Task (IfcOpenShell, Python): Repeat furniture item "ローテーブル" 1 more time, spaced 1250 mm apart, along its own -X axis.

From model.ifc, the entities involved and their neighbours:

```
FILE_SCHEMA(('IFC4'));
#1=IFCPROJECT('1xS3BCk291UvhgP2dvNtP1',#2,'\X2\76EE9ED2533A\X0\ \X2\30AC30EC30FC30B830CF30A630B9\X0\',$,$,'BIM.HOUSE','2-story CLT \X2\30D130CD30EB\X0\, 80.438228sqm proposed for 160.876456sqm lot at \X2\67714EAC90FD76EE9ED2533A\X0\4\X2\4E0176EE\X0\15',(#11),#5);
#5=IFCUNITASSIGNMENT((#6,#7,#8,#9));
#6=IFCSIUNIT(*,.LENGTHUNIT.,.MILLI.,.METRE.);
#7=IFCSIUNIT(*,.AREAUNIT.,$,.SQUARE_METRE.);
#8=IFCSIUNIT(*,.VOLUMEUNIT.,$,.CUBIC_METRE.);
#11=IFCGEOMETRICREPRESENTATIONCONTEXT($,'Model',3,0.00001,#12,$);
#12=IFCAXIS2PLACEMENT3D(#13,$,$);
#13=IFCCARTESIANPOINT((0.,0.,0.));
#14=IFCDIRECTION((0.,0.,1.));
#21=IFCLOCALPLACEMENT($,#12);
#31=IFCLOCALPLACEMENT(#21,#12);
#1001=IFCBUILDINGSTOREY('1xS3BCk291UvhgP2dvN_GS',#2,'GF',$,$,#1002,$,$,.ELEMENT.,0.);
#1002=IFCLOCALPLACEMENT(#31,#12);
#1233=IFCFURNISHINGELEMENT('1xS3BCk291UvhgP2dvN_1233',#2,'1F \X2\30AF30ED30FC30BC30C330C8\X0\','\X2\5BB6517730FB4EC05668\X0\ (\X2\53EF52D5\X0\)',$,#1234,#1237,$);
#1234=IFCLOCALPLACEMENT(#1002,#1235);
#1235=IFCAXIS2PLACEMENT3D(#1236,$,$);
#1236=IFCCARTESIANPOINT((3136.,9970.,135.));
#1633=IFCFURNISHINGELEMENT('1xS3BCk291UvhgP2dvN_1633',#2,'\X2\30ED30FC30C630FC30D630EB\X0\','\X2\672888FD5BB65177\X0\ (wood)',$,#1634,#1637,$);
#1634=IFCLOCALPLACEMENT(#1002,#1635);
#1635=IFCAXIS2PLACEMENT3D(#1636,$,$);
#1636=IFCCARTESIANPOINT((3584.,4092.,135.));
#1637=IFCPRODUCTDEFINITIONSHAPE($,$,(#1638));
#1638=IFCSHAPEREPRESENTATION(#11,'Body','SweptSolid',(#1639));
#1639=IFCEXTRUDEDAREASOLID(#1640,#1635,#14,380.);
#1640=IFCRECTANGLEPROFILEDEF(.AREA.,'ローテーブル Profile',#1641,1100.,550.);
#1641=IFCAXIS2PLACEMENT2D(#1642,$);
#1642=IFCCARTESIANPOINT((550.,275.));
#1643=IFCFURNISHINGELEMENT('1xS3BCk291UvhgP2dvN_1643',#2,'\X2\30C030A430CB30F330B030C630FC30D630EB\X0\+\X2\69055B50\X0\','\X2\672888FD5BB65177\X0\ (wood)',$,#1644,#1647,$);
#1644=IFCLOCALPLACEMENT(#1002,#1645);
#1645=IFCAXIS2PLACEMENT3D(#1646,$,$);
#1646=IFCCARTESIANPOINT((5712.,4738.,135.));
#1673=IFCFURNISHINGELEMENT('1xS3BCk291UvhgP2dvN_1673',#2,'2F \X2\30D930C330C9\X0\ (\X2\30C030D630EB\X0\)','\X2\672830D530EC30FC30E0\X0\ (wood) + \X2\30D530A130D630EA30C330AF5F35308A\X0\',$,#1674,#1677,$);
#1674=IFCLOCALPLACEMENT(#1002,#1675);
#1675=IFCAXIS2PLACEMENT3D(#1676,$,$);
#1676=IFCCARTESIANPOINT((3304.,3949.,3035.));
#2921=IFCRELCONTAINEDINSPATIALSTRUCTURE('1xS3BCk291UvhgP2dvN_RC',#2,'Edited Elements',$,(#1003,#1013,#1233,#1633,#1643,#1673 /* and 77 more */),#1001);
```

```python
import ifcopenshell
import ifcopenshell.api.geometry
import ifcopenshell.api.root
import ifcopenshell.util.element
import ifcopenshell.util.placement
import ifcopenshell.util.unit

model = ifcopenshell.open("model.ifc")
unit_scale = ifcopenshell.util.unit.calculate_unit_scale(model)


def reuse_history(source, copy):
    """copy_class also copies each property set's owner history, people and application; keep the originals."""
    for rel in copy.IsDefinedBy:
        if rel.is_a("IfcRelDefinesByProperties") and (history := rel.RelatingPropertyDefinition.OwnerHistory):
            rel.RelatingPropertyDefinition.OwnerHistory = source.OwnerHistory
            ifcopenshell.util.element.remove_deep2(model, history)


source = model.by_guid("1xS3BCk291UvhgP2dvN_1633")
base = ifcopenshell.util.placement.get_local_placement(source.ObjectPlacement)
step = -base[:3, 0] * 1.25 / unit_scale

for i in range(1, 2):
    copy = ifcopenshell.api.root.copy_class(model, product=source)
    copy.Representation = ifcopenshell.util.element.copy_deep(
        model, source.Representation, exclude=["IfcGeometricRepresentationContext", "IfcRepresentationMap"]
    )
    reuse_history(source, copy)
    matrix = base.copy()
    matrix[:3, 3] += i * step
    print("added at", matrix[:3, 3].round(3) + 0.0)
    ifcopenshell.api.geometry.edit_object_placement(model, product=copy, matrix=matrix, is_si=False)

model.write("model-out.ifc")
```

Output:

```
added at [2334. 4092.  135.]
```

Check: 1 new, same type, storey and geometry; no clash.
